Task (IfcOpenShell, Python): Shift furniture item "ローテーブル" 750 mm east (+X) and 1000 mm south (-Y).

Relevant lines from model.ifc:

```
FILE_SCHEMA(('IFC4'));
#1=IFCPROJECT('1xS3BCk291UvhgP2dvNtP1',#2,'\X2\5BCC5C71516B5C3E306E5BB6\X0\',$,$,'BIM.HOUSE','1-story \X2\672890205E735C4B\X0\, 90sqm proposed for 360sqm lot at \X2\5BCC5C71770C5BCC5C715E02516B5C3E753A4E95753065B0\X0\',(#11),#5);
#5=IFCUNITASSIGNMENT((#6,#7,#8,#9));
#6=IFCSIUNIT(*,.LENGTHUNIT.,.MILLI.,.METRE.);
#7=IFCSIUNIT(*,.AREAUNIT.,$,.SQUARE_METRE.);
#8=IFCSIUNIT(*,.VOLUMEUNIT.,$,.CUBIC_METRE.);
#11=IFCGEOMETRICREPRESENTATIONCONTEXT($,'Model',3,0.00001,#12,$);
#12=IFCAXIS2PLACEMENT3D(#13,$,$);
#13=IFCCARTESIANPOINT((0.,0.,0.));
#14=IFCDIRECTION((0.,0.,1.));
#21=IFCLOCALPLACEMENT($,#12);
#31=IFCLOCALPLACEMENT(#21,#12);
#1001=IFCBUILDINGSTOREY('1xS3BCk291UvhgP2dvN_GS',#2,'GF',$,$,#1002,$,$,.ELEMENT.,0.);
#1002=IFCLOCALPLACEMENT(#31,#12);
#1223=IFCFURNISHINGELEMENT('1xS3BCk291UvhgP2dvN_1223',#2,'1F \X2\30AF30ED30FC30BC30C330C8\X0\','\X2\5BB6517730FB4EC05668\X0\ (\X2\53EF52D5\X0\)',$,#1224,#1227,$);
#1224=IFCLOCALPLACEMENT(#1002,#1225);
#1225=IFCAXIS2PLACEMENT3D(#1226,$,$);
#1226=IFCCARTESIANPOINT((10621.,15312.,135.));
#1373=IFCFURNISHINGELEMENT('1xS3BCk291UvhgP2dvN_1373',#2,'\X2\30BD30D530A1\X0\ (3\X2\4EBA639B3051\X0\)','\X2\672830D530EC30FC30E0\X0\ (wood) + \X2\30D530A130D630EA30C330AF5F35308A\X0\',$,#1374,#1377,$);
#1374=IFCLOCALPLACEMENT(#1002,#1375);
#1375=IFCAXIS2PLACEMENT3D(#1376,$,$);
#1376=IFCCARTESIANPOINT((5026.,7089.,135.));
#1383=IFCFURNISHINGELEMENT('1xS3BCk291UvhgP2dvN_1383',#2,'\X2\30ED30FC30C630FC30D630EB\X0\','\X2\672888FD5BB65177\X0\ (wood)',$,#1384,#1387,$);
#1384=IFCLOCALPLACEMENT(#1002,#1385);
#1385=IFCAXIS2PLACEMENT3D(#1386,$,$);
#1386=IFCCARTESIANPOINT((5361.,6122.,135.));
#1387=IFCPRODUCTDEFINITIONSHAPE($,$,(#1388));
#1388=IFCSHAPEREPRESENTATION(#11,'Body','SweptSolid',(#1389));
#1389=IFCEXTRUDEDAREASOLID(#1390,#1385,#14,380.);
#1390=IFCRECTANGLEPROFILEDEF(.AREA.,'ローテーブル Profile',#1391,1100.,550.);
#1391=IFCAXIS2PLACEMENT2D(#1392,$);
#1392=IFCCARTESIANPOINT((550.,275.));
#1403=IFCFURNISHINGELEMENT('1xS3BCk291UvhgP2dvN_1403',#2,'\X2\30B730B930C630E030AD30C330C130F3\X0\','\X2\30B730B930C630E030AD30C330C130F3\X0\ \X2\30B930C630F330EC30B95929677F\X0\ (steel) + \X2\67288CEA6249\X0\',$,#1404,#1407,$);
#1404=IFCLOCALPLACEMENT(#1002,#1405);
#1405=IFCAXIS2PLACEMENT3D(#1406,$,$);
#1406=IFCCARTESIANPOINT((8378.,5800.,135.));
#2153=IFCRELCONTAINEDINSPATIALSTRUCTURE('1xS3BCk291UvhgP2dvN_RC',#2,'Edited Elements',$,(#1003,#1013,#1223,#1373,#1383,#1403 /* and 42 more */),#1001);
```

```python
import ifcopenshell
import ifcopenshell.api.geometry
import ifcopenshell.util.placement
import ifcopenshell.util.unit

model = ifcopenshell.open("model.ifc")
unit_scale = ifcopenshell.util.unit.calculate_unit_scale(model)

item = model.by_guid("1xS3BCk291UvhgP2dvN_1383")
matrix = ifcopenshell.util.placement.get_local_placement(item.ObjectPlacement)
matrix[0, 3] += 0.75 / unit_scale
matrix[1, 3] -= 1 / unit_scale
ifcopenshell.api.geometry.edit_object_placement(model, product=item, matrix=matrix, is_si=False)

print(ifcopenshell.util.placement.get_local_placement(item.ObjectPlacement).round(3) + 0.0)

model.write("model-out.ifc")
```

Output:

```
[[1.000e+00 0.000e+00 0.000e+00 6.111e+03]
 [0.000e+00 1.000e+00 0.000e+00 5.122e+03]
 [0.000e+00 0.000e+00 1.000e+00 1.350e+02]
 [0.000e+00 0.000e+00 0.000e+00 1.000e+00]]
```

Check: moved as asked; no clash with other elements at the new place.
